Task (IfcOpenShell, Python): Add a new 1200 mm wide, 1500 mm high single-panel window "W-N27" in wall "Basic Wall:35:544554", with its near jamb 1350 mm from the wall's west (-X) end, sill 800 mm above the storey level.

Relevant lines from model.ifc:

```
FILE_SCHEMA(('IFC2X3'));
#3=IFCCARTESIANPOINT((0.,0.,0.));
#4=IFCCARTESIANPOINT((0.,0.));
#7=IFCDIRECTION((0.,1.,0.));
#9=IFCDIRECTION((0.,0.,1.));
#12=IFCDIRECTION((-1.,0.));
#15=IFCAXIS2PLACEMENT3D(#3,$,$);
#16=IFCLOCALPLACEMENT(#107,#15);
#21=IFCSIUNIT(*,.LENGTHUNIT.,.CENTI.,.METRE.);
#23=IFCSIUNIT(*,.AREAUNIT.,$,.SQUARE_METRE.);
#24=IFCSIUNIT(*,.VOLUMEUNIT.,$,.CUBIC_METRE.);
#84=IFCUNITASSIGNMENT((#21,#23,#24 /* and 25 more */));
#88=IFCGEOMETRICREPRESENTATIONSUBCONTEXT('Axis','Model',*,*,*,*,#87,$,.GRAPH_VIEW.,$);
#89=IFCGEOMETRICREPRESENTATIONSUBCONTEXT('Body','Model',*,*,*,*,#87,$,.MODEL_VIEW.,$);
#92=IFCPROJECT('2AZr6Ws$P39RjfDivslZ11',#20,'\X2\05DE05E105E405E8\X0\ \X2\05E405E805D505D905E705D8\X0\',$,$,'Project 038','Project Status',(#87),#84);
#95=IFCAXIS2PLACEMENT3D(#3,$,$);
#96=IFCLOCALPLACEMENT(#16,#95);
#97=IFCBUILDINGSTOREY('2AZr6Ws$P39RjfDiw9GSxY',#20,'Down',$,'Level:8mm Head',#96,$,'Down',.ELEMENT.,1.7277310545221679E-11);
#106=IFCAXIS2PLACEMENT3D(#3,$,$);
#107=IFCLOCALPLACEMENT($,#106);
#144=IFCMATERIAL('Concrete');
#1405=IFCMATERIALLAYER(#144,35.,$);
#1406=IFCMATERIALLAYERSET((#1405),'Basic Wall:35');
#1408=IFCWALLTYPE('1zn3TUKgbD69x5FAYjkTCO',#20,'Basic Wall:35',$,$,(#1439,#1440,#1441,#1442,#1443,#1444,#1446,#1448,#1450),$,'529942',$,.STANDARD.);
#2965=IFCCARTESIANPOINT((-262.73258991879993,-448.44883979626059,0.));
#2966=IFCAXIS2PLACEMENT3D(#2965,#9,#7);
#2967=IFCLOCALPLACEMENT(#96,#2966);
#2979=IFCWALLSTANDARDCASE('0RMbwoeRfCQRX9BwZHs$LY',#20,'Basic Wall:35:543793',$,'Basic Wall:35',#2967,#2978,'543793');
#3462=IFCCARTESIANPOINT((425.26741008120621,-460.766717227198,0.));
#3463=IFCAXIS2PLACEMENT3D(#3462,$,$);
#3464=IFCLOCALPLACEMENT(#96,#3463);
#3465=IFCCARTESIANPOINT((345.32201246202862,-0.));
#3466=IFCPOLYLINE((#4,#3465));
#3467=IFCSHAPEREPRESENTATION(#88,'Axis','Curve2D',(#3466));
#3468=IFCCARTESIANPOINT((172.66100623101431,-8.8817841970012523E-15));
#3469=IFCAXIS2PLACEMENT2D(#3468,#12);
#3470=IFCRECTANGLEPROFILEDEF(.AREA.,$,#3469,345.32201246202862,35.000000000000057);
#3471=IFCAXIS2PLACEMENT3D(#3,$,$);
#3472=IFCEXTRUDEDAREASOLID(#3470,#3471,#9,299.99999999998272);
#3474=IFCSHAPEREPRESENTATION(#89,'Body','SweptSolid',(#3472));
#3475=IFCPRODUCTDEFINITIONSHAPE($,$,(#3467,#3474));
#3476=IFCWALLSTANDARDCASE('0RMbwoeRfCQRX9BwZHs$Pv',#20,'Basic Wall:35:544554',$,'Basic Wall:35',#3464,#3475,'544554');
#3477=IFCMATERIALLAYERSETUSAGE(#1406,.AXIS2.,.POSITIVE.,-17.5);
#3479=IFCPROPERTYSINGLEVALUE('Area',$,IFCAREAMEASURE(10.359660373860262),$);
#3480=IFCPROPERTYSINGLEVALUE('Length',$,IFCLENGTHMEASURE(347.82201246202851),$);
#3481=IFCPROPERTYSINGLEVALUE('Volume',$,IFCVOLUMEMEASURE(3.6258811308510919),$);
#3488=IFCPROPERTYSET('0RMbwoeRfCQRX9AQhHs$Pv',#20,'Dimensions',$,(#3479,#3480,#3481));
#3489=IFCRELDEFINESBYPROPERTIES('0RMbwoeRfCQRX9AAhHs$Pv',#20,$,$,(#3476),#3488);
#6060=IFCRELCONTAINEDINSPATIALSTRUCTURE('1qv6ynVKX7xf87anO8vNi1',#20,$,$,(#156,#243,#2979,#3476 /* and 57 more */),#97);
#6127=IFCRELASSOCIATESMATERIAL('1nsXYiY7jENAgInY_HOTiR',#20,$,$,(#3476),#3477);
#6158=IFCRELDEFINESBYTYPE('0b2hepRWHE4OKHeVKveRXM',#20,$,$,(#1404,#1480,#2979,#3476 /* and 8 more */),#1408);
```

```python
import numpy as np
import ifcopenshell
import ifcopenshell.api.feature
import ifcopenshell.api.geometry
import ifcopenshell.api.pset
import ifcopenshell.api.root
import ifcopenshell.api.spatial
import ifcopenshell.api.type
import ifcopenshell.geom
import ifcopenshell.util.element
import ifcopenshell.util.placement
import ifcopenshell.util.representation
import ifcopenshell.util.shape
import ifcopenshell.util.unit

model = ifcopenshell.open("model.ifc")
unit_scale = ifcopenshell.util.unit.calculate_unit_scale(model)
area_scale = ifcopenshell.util.unit.calculate_unit_scale(model, "AREAUNIT")
volume_scale = ifcopenshell.util.unit.calculate_unit_scale(model, "VOLUMEUNIT")
settings = ifcopenshell.geom.settings()


def volume(element):
    """Net volume in cubic metres, openings subtracted."""
    shape = ifcopenshell.geom.create_shape(settings, element)
    return ifcopenshell.util.shape.get_volume(shape.geometry)


wall = model.by_guid("0RMbwoeRfCQRX9BwZHs$Pv")
storey = ifcopenshell.util.element.get_container(wall, ifc_class="IfcBuildingStorey")
context = ifcopenshell.util.representation.get_context(model, "Model", "Body", "MODEL_VIEW")
before = volume(wall)

width, height, from_end, sill = 1.2, 1.5, 1.35, 0.8  # metres

# The wall runs along its own X axis, and the end named is its -X end.
wall_shape = ifcopenshell.geom.create_shape(settings, wall)
x, y, z = ifcopenshell.util.shape.get_vertices(wall_shape.geometry).T
start = x.min() + from_end
face, thickness = float(y.min()), float(y.max() - y.min())
wall_matrix = ifcopenshell.util.placement.get_local_placement(wall.ObjectPlacement)
level = ifcopenshell.util.placement.get_local_placement(storey.ObjectPlacement)[2, 3]


def in_wall(x, y):
    """Placement at x, y metres in the wall's axes, at sill height."""
    matrix = wall_matrix.copy()
    matrix[:, 3] = wall_matrix @ np.array([x / unit_scale, y / unit_scale, 0.0, 1.0])
    matrix[2, 3] = level + sill / unit_scale
    return matrix


# Opening: a box that overshoots both wall faces by 50 mm.
opening = ifcopenshell.api.root.create_entity(model, ifc_class="IfcOpeningElement")
box = ifcopenshell.api.geometry.add_wall_representation(
    model, context=context, length=width, height=height, thickness=thickness + 0.1
)
ifcopenshell.api.geometry.assign_representation(model, product=opening, representation=box)
ifcopenshell.api.geometry.edit_object_placement(model, product=opening, matrix=in_wall(start, face - 0.05), is_si=False)
ifcopenshell.api.feature.add_feature(model, feature=opening, element=wall)

window = ifcopenshell.api.root.create_entity(model, ifc_class="IfcWindow", name="W-N27")
window.OverallWidth, window.OverallHeight = width / unit_scale, height / unit_scale
body = ifcopenshell.api.geometry.add_window_representation(
    model,
    context=context,
    overall_width=window.OverallWidth,
    overall_height=window.OverallHeight,
    partition_type="SINGLE_PANEL",
)
ifcopenshell.api.geometry.assign_representation(model, product=window, representation=body)
ifcopenshell.api.spatial.assign_container(model, products=[window], relating_structure=storey)
fills = ifcopenshell.api.feature.add_filling(model, opening=opening, element=window)
fills.OwnerHistory = window.OwnerHistory  # required in IFC2X3

# IFC2X3 keeps the operation on the window style.
style = ifcopenshell.api.root.create_entity(model, ifc_class="IfcWindowStyle", name="W-N27")
style.OperationType, style.ConstructionType = "SINGLE_PANEL", "NOTDEFINED"
style.ParameterTakesPrecedence = style.Sizeable = False
ifcopenshell.api.type.assign_type(model, related_objects=[window], relating_type=style)

# Centre the window in the wall's thickness.
ifcopenshell.api.geometry.edit_object_placement(model, product=window, matrix=in_wall(start, face), is_si=False)
window_shape = ifcopenshell.geom.create_shape(settings, window)
depth = ifcopenshell.util.shape.get_vertices(window_shape.geometry)[:, 1]
offset = face + thickness / 2 - (depth.min() + depth.max()) / 2
ifcopenshell.api.geometry.edit_object_placement(model, product=window, matrix=in_wall(start, offset), is_si=False)

after = volume(wall)

# Update the wall's stored quantities.
pset = model.by_id(ifcopenshell.util.element.get_pset(wall, "Dimensions", should_inherit=False)["id"])
ifcopenshell.api.pset.edit_pset(model, pset=pset, properties={
    "Area": model.create_entity("IfcAreaMeasure", after / thickness / area_scale),
    "Volume": model.create_entity("IfcVolumeMeasure", after / volume_scale),
})

print(f"wall volume {before:.3f} -> {after:.3f} m3")

model.write("model_updated.ifc")
```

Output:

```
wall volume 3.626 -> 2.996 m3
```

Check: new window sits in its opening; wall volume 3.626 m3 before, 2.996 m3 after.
